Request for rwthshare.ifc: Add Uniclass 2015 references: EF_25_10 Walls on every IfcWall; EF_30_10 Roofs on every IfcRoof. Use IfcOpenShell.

First a look at what the model holds.

```python
import ifcopenshell

model = ifcopenshell.open("rwthshare.ifc")
print(model.schema)
print("classifications:", [c.Name for c in model.by_type("IfcClassification")])
for ifc_class in ("IfcDoor", "IfcRoof", "IfcStair", "IfcWall", "IfcWindow"):
    print(ifc_class, len(model.by_type(ifc_class)))
```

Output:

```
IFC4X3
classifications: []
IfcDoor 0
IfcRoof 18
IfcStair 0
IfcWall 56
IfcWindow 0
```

```python
import ifcopenshell
import ifcopenshell.api.classification

model = ifcopenshell.open("rwthshare.ifc")

system = ifcopenshell.api.classification.add_classification(model, classification="Uniclass 2015")

codes = {
    "IfcWall": ("EF_25_10", "Walls"),
    "IfcRoof": ("EF_30_10", "Roofs"),
}
for ifc_class, (code, name) in codes.items():
    products = model.by_type(ifc_class)
    ifcopenshell.api.classification.add_reference(
        model, products=products, classification=system, identification=code, name=name
    )
    print(code, len(products))

model.write("rwthshare_edited.ifc")
```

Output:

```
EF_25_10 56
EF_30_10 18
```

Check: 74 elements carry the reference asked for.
